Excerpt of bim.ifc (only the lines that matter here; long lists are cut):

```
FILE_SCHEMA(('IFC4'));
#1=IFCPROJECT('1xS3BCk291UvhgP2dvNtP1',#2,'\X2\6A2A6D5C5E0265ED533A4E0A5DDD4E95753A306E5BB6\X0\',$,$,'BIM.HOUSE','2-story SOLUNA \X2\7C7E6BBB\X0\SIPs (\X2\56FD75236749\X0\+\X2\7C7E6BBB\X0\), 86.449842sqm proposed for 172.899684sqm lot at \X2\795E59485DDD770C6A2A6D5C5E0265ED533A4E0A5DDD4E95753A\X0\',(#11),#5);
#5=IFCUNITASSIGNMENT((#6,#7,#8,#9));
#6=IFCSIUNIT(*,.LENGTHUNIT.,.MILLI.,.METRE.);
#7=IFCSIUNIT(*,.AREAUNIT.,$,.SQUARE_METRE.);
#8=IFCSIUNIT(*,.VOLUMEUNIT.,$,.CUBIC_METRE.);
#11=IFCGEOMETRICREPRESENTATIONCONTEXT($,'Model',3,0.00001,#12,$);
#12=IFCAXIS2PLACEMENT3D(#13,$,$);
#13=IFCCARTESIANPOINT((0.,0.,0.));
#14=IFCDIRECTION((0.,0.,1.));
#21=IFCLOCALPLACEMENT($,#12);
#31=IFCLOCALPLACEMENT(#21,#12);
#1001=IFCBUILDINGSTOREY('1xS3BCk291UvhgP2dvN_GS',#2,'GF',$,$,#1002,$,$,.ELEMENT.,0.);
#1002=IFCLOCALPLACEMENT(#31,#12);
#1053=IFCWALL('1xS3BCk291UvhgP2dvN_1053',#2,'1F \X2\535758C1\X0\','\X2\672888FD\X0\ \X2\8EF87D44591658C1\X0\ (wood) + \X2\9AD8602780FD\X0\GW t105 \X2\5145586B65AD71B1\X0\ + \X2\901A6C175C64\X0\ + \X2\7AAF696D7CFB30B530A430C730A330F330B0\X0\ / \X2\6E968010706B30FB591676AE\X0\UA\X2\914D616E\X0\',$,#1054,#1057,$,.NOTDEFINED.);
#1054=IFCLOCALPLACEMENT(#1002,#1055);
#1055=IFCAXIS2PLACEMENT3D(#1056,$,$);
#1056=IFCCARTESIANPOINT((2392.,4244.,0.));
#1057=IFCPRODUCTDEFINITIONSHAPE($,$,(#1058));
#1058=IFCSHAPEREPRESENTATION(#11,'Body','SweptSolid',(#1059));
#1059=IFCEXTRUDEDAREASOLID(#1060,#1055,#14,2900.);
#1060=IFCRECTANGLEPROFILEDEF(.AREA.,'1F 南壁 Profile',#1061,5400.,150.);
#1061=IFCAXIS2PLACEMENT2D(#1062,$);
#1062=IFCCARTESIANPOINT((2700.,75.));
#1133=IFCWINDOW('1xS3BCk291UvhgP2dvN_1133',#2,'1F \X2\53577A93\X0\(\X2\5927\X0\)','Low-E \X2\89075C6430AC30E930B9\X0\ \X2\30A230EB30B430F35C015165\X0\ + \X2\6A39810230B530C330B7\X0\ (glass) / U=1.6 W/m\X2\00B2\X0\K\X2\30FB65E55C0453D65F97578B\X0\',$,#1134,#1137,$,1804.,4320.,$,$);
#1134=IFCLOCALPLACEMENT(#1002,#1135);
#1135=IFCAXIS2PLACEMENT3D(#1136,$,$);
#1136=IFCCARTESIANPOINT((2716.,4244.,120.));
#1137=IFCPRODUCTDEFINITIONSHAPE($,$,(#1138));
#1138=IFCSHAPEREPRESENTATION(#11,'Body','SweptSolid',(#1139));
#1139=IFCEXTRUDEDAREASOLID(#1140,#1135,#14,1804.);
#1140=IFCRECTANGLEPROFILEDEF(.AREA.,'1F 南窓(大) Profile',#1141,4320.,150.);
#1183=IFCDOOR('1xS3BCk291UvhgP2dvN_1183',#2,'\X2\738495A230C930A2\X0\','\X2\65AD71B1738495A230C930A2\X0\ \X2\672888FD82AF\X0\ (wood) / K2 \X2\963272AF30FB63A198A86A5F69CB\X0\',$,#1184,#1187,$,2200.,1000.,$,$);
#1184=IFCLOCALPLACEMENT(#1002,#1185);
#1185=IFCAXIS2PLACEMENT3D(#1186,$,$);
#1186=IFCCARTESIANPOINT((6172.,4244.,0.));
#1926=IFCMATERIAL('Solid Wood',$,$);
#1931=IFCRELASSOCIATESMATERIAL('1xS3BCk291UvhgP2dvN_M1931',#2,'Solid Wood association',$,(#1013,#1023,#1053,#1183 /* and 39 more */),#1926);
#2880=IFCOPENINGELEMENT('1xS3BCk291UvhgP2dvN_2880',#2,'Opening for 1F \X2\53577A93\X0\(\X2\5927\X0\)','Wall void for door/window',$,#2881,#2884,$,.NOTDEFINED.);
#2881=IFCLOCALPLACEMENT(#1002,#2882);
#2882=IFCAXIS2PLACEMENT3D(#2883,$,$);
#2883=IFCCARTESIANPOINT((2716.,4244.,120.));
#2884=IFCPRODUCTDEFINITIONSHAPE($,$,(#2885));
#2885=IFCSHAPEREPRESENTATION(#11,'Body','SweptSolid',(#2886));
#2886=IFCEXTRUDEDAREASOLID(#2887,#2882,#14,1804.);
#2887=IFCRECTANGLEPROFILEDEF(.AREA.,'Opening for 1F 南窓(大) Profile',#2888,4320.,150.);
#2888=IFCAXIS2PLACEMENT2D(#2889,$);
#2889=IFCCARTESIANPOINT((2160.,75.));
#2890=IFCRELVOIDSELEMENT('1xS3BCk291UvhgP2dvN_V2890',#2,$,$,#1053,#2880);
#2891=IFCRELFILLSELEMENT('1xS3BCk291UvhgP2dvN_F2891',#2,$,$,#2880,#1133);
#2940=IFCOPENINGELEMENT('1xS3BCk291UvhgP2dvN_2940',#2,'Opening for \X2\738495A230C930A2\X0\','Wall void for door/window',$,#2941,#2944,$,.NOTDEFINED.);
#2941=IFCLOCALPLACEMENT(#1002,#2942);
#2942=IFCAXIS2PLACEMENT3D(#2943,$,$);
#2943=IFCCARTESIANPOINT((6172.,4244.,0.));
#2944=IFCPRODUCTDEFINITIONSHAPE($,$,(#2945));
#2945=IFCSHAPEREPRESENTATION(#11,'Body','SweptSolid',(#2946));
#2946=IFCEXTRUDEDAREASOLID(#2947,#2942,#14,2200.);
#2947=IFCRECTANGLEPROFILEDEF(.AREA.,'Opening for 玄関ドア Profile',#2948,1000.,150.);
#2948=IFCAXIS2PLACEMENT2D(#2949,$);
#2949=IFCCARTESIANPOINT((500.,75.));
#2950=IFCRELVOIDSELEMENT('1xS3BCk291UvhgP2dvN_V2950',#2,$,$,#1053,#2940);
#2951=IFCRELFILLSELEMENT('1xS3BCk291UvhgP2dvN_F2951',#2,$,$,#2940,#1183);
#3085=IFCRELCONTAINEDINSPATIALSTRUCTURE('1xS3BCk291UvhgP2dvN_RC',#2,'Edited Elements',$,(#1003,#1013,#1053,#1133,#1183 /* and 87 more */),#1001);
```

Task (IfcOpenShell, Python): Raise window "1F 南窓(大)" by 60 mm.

```python
import numpy as np
import ifcopenshell
import ifcopenshell.api.geometry
import ifcopenshell.util.placement
import ifcopenshell.util.unit

model = ifcopenshell.open("bim.ifc")
unit_scale = ifcopenshell.util.unit.calculate_unit_scale(model)

window = model.by_guid("1xS3BCk291UvhgP2dvN_1133")
opening = window.FillsVoids[0].RelatingOpeningElement
dz = 60.0

shift = np.array([0.0, 0.0, dz])
# The window is not placed relative to its opening, so move both.
for product in (opening, window):
    matrix = ifcopenshell.util.placement.get_local_placement(product.ObjectPlacement)
    matrix[:3, 3] += shift
    ifcopenshell.api.geometry.edit_object_placement(model, product=product, matrix=matrix, is_si=False)

print(f"moved by {dz * unit_scale:+.3f} m")

model.write("bim_v2.ifc")
```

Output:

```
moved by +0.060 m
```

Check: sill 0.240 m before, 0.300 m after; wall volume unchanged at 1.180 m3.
